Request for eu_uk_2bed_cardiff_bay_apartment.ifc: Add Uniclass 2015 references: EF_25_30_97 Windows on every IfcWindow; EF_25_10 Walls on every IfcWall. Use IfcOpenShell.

First a look at what the model holds.

```python
import ifcopenshell

model = ifcopenshell.open("eu_uk_2bed_cardiff_bay_apartment.ifc")
print(model.schema)
print("classifications:", [c.Name for c in model.by_type("IfcClassification")])
for ifc_class in ("IfcDoor", "IfcRoof", "IfcStair", "IfcWall", "IfcWindow"):
    print(ifc_class, len(model.by_type(ifc_class)))
```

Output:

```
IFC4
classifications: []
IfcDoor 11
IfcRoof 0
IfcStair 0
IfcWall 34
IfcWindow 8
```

```python
import ifcopenshell
import ifcopenshell.api.classification

model = ifcopenshell.open("eu_uk_2bed_cardiff_bay_apartment.ifc")

system = ifcopenshell.api.classification.add_classification(model, classification="Uniclass 2015")

codes = {
    "IfcWindow": ("EF_25_30_97", "Windows"),
    "IfcWall": ("EF_25_10", "Walls"),
}
for ifc_class, (code, name) in codes.items():
    products = model.by_type(ifc_class)
    ifcopenshell.api.classification.add_reference(
        model, products=products, classification=system, identification=code, name=name
    )
    print(code, len(products))

model.write("eu_uk_2bed_cardiff_bay_apartment_edited.ifc")
```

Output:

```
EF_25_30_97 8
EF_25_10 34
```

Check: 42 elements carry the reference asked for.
